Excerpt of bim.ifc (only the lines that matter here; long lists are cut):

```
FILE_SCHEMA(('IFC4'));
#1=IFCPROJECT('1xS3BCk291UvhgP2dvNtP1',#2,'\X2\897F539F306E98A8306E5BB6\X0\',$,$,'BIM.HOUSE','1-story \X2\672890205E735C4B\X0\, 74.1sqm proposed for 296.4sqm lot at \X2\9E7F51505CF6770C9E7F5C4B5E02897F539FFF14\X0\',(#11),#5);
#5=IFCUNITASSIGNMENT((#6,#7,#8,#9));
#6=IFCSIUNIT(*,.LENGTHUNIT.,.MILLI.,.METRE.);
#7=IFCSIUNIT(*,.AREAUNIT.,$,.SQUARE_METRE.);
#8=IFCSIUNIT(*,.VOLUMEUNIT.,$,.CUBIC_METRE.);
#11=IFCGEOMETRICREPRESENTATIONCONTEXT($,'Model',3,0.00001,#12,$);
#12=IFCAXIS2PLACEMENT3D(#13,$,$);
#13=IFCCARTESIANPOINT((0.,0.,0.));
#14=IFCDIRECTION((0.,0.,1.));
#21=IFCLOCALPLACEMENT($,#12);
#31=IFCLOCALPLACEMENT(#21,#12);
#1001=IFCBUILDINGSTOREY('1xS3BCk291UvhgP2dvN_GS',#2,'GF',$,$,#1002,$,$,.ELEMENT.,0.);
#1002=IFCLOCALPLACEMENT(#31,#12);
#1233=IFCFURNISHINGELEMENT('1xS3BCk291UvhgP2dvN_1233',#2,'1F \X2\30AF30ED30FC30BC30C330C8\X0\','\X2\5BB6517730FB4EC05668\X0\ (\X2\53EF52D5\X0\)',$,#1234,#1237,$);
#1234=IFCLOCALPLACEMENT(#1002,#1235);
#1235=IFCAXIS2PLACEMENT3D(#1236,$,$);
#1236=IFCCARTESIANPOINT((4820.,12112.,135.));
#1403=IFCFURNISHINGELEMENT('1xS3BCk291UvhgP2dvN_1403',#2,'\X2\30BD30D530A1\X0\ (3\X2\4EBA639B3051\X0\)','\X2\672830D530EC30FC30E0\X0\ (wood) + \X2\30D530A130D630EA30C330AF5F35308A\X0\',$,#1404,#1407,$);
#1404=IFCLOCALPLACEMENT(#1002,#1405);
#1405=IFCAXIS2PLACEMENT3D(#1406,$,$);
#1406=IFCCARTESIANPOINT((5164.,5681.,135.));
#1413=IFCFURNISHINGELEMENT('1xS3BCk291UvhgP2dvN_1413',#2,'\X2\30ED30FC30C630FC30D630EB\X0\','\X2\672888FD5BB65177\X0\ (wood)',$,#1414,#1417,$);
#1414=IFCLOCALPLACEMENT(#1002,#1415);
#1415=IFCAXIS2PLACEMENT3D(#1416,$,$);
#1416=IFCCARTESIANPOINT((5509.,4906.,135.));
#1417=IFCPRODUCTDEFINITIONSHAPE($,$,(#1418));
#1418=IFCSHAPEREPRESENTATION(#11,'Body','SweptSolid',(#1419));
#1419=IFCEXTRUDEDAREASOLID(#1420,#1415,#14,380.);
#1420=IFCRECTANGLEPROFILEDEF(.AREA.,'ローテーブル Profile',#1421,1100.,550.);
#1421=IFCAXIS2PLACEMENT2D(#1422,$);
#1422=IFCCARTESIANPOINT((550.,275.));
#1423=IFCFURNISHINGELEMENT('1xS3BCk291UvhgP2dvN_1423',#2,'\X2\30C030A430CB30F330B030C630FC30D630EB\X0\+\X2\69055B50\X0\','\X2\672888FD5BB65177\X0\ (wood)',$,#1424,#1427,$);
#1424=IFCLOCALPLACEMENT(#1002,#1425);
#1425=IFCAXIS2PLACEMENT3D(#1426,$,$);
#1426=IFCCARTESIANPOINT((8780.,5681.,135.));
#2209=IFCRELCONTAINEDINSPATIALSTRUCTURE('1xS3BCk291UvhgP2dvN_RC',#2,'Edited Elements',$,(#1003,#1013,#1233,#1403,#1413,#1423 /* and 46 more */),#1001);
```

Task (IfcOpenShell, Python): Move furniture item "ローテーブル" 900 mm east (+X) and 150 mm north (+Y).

```python
import ifcopenshell
import ifcopenshell.api.geometry
import ifcopenshell.util.placement
import ifcopenshell.util.unit

model = ifcopenshell.open("bim.ifc")
unit_scale = ifcopenshell.util.unit.calculate_unit_scale(model)

item = model.by_guid("1xS3BCk291UvhgP2dvN_1413")
matrix = ifcopenshell.util.placement.get_local_placement(item.ObjectPlacement)
matrix[0, 3] += 0.9 / unit_scale
matrix[1, 3] += 0.15 / unit_scale
ifcopenshell.api.geometry.edit_object_placement(model, product=item, matrix=matrix, is_si=False)

print(ifcopenshell.util.placement.get_local_placement(item.ObjectPlacement).round(3) + 0.0)

model.write("bim_v2.ifc")
```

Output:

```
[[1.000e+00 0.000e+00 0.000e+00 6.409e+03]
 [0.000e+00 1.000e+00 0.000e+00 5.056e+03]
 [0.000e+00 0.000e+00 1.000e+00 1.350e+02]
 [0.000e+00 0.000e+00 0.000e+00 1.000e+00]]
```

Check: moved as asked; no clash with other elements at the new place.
